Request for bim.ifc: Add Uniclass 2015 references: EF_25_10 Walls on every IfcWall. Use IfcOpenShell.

First a look at what the model holds.

```python
import ifcopenshell

model = ifcopenshell.open("bim.ifc")
print(model.schema)
print("classifications:", [c.Name for c in model.by_type("IfcClassification")])
for ifc_class in ("IfcDoor", "IfcRoof", "IfcStair", "IfcWall", "IfcWindow"):
    print(ifc_class, len(model.by_type(ifc_class)))
```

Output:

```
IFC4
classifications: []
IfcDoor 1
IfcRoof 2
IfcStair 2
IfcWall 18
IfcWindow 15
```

```python
import ifcopenshell
import ifcopenshell.api.classification

model = ifcopenshell.open("bim.ifc")

system = ifcopenshell.api.classification.add_classification(model, classification="Uniclass 2015")

codes = {
    "IfcWall": ("EF_25_10", "Walls"),
}
for ifc_class, (code, name) in codes.items():
    products = model.by_type(ifc_class)
    ifcopenshell.api.classification.add_reference(
        model, products=products, classification=system, identification=code, name=name
    )
    print(code, len(products))

model.write("bim-out.ifc")
```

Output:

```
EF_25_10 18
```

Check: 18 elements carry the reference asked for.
